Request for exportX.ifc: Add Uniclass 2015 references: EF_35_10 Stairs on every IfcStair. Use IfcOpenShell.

First a look at what the model holds.

```python
import ifcopenshell

model = ifcopenshell.open("exportX.ifc")
print(model.schema)
print("classifications:", [c.Name for c in model.by_type("IfcClassification")])
for ifc_class in ("IfcDoor", "IfcRoof", "IfcStair", "IfcWall", "IfcWindow"):
    print(ifc_class, len(model.by_type(ifc_class)))
```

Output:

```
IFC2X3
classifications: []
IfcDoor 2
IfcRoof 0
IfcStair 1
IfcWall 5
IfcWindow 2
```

```python
import ifcopenshell
import ifcopenshell.api.classification

model = ifcopenshell.open("exportX.ifc")

# IFC2X3 requires Source and Edition and has no link from the project to the system.
system = model.create_entity("IfcClassification", Source="NBS", Edition="2015", Name="Uniclass 2015")

codes = {
    "IfcStair": ("EF_35_10", "Stairs"),
}
for ifc_class, (code, name) in codes.items():
    products = model.by_type(ifc_class)
    ifcopenshell.api.classification.add_reference(
        model, products=products, classification=system, identification=code, name=name
    )
    print(code, len(products))

model.write("exportX-out.ifc")
```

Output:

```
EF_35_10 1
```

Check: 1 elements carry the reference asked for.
